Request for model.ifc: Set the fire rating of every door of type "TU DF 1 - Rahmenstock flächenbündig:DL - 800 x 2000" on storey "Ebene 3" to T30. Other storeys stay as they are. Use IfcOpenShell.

First a look at what the model holds.

```python
import ifcopenshell
import ifcopenshell.util.element

model = ifcopenshell.open("model.ifc")
print(model.schema)
storey = next(s for s in model.by_type("IfcBuildingStorey") if s.Name == "Ebene 3")
doors = [e for e in ifcopenshell.util.element.get_decomposition(storey) if e.is_a("IfcDoor")]
seen = {}
for e in doors:
    element_type = ifcopenshell.util.element.get_type(e)
    key = (element_type.Name if element_type != e and element_type else None, ifcopenshell.util.element.get_pset(e, "Pset_DoorCommon", "FireRating"))
    seen[key] = seen.get(key, 0) + 1
for (name, value), count in sorted(seen.items(), key=str):
    print(count, "x", name, "|", value)
```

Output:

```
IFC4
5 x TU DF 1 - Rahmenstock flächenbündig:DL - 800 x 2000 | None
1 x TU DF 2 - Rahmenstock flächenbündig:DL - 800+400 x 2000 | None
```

```python
import ifcopenshell
import ifcopenshell.api.pset
import ifcopenshell.util.element

model = ifcopenshell.open("model.ifc")

storey = next(s for s in model.by_type("IfcBuildingStorey") if s.Name == "Ebene 3")
doors = [e for e in ifcopenshell.util.element.get_decomposition(storey) if e.is_a("IfcDoor")]

count = 0
for e in doors:
    element_type = ifcopenshell.util.element.get_type(e)
    if element_type in (None, e) or element_type.Name != "TU DF 1 - Rahmenstock flächenbündig:DL - 800 x 2000":
        continue
    # add_pset returns the element's existing set when there is one.
    pset = ifcopenshell.api.pset.add_pset(model, product=e, name="Pset_DoorCommon")
    ifcopenshell.api.pset.edit_pset(model, pset=pset, properties={"FireRating": "T30"})
    count += 1

print(count, "doors updated")

model.write("model_rev.ifc")
```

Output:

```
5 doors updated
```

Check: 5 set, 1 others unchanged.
